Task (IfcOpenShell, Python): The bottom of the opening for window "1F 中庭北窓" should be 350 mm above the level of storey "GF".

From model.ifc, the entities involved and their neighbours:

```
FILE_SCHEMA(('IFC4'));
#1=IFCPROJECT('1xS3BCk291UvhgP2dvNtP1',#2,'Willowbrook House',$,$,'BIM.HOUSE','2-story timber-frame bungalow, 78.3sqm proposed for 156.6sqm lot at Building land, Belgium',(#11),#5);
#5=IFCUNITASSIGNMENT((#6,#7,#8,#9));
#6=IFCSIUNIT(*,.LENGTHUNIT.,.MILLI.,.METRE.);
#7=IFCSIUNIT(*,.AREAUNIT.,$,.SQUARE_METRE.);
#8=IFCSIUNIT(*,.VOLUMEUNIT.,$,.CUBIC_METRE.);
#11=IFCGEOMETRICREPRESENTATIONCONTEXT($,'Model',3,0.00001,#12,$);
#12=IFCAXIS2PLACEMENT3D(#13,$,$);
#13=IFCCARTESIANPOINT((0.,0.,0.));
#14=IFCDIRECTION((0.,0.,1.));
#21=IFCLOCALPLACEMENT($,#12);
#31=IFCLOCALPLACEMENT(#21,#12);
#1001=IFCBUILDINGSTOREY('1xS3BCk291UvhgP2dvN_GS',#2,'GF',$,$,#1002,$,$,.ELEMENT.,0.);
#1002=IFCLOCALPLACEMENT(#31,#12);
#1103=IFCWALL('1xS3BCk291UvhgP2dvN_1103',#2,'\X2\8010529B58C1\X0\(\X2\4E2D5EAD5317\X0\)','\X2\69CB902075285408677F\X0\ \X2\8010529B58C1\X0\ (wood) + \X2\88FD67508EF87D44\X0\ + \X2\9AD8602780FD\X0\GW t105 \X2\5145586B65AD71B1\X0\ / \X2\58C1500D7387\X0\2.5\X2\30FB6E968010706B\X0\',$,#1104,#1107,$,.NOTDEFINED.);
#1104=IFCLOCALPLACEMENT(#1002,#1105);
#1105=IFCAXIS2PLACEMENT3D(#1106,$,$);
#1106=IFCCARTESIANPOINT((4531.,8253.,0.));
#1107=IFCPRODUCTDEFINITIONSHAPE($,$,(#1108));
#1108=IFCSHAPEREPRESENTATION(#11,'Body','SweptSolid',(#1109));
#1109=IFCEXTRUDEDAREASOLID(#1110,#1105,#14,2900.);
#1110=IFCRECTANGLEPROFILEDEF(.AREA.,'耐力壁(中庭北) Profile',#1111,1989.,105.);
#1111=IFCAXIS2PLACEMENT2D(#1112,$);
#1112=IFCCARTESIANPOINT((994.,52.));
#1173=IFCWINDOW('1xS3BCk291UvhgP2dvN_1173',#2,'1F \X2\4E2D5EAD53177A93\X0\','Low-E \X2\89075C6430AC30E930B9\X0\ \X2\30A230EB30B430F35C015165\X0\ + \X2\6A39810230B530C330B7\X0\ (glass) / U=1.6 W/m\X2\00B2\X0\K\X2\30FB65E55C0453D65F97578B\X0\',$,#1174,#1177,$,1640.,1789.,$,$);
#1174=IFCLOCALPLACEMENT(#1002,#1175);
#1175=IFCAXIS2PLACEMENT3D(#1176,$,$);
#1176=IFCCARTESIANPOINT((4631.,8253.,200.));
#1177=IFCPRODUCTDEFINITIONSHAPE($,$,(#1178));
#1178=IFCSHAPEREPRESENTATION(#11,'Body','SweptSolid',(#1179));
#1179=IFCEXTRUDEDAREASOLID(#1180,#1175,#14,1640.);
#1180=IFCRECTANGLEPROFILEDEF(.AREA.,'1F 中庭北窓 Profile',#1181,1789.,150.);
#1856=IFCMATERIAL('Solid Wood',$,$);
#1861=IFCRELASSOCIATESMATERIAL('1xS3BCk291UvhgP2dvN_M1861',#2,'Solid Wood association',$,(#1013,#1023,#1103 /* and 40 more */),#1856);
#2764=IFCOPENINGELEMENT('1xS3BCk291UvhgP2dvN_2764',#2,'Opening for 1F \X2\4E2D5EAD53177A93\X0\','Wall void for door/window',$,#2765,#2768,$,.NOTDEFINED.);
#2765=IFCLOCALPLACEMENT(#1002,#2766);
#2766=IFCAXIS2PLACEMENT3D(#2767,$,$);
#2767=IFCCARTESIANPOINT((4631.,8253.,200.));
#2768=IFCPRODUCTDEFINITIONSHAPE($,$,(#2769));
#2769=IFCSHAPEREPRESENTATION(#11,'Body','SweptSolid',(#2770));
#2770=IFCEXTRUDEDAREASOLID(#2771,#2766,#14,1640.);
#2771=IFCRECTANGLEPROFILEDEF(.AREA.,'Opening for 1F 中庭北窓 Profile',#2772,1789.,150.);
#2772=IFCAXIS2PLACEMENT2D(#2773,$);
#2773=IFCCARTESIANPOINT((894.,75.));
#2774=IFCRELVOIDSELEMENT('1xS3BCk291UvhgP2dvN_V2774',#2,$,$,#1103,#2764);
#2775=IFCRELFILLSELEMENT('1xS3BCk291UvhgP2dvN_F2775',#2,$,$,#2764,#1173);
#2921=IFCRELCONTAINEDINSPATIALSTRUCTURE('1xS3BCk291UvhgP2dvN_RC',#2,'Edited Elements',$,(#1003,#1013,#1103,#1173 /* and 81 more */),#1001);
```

```python
import numpy as np
import ifcopenshell
import ifcopenshell.api.geometry
import ifcopenshell.geom
import ifcopenshell.util.element
import ifcopenshell.util.placement
import ifcopenshell.util.shape
import ifcopenshell.util.unit

model = ifcopenshell.open("model.ifc")
unit_scale = ifcopenshell.util.unit.calculate_unit_scale(model)

window = model.by_guid("1xS3BCk291UvhgP2dvN_1173")
opening = window.FillsVoids[0].RelatingOpeningElement
storey = ifcopenshell.util.element.get_container(window, ifc_class="IfcBuildingStorey")
level = ifcopenshell.util.placement.get_local_placement(storey.ObjectPlacement)[2, 3]

# The opening's origin need not be at the sill, so measure its lowest point.
shape = ifcopenshell.geom.create_shape(ifcopenshell.geom.settings(), opening)
bottom = ifcopenshell.util.shape.get_shape_bottom_elevation(shape, shape.geometry) / unit_scale
dz = level + 0.35 / unit_scale - bottom

shift = np.array([0.0, 0.0, dz])
# The window is not placed relative to its opening, so move both.
for product in (opening, window):
    matrix = ifcopenshell.util.placement.get_local_placement(product.ObjectPlacement)
    matrix[:3, 3] += shift
    ifcopenshell.api.geometry.edit_object_placement(model, product=product, matrix=matrix, is_si=False)

print(f"moved by {dz * unit_scale:+.3f} m")

model.write("model_v2.ifc")
```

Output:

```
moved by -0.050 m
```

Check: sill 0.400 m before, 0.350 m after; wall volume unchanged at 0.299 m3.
